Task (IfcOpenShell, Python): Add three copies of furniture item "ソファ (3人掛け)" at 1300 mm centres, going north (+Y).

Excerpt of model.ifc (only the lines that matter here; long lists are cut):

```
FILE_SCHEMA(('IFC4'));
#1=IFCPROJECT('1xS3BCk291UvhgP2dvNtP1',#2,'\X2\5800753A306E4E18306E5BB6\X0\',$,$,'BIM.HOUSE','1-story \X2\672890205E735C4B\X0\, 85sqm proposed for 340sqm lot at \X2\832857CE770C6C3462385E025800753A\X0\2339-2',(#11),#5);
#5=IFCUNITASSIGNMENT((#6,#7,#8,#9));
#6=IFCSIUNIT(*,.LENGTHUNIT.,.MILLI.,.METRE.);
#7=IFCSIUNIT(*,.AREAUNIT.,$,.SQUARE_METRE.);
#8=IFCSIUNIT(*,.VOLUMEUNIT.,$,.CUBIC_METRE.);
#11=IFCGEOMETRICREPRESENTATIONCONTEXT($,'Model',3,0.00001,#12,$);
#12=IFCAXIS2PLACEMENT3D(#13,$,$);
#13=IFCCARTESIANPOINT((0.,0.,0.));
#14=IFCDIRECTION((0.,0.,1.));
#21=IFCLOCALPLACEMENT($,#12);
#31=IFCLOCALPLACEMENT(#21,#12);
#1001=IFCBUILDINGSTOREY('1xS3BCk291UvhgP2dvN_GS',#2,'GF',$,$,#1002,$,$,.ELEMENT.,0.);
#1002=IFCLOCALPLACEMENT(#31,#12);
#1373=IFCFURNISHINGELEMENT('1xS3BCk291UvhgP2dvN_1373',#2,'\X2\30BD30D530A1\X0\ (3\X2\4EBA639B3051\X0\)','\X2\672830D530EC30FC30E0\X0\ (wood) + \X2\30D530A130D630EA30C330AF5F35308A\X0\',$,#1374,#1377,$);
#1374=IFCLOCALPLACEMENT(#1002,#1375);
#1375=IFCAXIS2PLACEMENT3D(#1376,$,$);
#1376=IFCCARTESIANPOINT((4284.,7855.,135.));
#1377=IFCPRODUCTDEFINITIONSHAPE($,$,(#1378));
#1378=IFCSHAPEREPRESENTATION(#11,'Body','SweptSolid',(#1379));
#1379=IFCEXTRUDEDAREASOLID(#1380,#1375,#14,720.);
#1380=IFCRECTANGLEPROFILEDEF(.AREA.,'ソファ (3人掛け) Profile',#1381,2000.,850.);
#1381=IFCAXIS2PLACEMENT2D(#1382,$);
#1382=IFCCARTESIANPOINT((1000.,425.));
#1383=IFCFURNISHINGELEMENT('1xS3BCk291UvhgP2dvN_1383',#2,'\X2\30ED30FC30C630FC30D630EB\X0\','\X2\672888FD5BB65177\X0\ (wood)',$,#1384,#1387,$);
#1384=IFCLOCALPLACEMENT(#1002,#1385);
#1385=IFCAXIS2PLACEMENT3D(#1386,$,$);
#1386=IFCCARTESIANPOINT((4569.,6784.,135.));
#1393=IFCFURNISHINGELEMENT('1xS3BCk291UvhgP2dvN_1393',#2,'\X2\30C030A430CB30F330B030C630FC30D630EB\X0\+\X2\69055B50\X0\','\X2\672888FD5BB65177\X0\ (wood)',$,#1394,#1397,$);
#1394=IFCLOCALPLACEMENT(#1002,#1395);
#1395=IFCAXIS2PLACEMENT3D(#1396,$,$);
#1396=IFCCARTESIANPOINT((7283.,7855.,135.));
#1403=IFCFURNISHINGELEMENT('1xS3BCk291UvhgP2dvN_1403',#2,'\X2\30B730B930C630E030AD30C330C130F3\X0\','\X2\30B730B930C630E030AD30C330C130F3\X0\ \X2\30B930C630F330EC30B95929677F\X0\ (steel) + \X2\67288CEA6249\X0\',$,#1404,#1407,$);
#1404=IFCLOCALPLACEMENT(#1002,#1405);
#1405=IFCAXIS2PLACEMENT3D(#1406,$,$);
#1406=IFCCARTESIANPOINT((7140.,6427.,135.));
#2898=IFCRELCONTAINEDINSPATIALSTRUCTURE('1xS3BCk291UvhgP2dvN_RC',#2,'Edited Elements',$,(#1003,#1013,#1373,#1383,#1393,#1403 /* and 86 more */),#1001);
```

```python
import numpy as np
import ifcopenshell
import ifcopenshell.api.geometry
import ifcopenshell.api.root
import ifcopenshell.util.element
import ifcopenshell.util.placement
import ifcopenshell.util.unit

model = ifcopenshell.open("model.ifc")
unit_scale = ifcopenshell.util.unit.calculate_unit_scale(model)


def reuse_history(source, copy):
    """copy_class also copies each property set's owner history, people and application; keep the originals."""
    for rel in copy.IsDefinedBy:
        if rel.is_a("IfcRelDefinesByProperties") and (history := rel.RelatingPropertyDefinition.OwnerHistory):
            rel.RelatingPropertyDefinition.OwnerHistory = source.OwnerHistory
            ifcopenshell.util.element.remove_deep2(model, history)


source = model.by_guid("1xS3BCk291UvhgP2dvN_1373")
base = ifcopenshell.util.placement.get_local_placement(source.ObjectPlacement)
step = np.array([0.0, 1.0, 0.0]) * 1.3 / unit_scale

for i in range(1, 4):
    copy = ifcopenshell.api.root.copy_class(model, product=source)
    copy.Representation = ifcopenshell.util.element.copy_deep(
        model, source.Representation, exclude=["IfcGeometricRepresentationContext", "IfcRepresentationMap"]
    )
    reuse_history(source, copy)
    matrix = base.copy()
    matrix[:3, 3] += i * step
    print("added at", matrix[:3, 3].round(3) + 0.0)
    ifcopenshell.api.geometry.edit_object_placement(model, product=copy, matrix=matrix, is_si=False)

model.write("model_rev.ifc")
```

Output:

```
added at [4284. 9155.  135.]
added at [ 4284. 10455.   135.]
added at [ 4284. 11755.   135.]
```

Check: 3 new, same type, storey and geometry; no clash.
